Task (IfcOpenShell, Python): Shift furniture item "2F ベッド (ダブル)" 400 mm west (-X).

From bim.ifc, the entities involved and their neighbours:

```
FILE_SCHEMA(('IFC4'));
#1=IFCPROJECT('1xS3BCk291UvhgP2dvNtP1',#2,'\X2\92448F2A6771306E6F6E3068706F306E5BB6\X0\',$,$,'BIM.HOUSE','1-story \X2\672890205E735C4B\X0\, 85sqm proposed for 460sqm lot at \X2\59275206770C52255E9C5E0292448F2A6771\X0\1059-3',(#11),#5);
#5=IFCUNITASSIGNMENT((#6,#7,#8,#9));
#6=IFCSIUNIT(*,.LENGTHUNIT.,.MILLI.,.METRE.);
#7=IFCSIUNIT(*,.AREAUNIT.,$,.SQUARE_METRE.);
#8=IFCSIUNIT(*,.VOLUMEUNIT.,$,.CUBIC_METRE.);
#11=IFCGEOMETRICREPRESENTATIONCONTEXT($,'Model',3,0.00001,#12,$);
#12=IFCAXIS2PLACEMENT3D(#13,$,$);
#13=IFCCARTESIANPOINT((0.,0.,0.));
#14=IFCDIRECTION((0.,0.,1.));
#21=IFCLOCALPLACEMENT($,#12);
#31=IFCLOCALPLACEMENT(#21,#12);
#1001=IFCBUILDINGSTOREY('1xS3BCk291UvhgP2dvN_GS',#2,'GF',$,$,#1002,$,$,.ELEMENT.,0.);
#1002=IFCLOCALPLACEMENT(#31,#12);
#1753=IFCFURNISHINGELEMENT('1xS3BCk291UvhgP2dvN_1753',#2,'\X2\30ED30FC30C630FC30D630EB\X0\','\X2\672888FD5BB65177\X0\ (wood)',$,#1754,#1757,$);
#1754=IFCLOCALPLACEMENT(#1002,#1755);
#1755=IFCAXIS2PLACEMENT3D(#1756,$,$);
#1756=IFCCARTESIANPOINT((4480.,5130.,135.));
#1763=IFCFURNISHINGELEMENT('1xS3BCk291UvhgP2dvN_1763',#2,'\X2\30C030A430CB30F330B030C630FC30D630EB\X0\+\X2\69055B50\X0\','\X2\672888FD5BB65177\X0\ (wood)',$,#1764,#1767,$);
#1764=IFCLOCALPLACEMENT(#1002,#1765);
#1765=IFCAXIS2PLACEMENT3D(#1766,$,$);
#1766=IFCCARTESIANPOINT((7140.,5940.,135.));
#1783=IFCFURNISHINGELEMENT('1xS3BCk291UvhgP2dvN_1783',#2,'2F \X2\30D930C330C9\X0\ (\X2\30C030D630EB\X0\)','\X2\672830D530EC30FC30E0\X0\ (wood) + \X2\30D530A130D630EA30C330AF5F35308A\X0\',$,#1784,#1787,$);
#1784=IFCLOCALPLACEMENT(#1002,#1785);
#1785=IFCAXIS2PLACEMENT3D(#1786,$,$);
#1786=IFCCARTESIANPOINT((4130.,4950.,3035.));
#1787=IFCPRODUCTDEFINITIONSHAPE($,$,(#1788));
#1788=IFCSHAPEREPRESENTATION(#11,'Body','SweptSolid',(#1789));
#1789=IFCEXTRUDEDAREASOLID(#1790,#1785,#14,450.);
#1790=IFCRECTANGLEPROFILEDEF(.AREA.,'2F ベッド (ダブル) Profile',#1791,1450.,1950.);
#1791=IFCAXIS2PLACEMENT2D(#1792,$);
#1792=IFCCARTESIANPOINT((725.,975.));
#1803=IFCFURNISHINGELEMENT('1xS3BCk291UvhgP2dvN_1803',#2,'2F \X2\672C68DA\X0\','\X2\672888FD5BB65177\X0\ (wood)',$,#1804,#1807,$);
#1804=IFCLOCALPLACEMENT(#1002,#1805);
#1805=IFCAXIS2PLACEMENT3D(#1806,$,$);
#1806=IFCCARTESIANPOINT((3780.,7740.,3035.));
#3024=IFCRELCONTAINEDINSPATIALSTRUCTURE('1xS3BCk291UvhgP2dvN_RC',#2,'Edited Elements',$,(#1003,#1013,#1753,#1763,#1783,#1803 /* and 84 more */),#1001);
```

```python
import ifcopenshell
import ifcopenshell.api.geometry
import ifcopenshell.util.placement

model = ifcopenshell.open("bim.ifc")

item = model.by_id(1783)
matrix = ifcopenshell.util.placement.get_local_placement(item.ObjectPlacement)
matrix[0, 3] -= 400.0
ifcopenshell.api.geometry.edit_object_placement(model, product=item, matrix=matrix, is_si=False)

print(ifcopenshell.util.placement.get_local_placement(item.ObjectPlacement).round(3) + 0.0)

model.write("bim_v2.ifc")
```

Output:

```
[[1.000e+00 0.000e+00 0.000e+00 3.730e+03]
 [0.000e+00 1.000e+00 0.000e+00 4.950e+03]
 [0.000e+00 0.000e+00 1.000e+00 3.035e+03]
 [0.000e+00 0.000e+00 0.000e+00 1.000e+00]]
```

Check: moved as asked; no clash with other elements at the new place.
